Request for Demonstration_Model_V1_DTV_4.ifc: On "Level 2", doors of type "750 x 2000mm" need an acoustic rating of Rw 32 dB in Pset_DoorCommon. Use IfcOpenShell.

First a look at what the model holds.

```python
import ifcopenshell
import ifcopenshell.util.element

model = ifcopenshell.open("Demonstration_Model_V1_DTV_4.ifc")
print(model.schema)
storey = next(s for s in model.by_type("IfcBuildingStorey") if s.Name == "Level 2")
doors = [e for e in ifcopenshell.util.element.get_decomposition(storey) if e.is_a("IfcDoor")]
seen = {}
for e in doors:
    element_type = ifcopenshell.util.element.get_type(e)
    key = (element_type.Name if element_type != e and element_type else None, ifcopenshell.util.element.get_pset(e, "Pset_DoorCommon", "AcousticRating"))
    seen[key] = seen.get(key, 0) + 1
for (name, value), count in sorted(seen.items(), key=str):
    print(count, "x", name, "|", value)
```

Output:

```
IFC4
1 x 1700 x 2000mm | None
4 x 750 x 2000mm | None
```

```python
import ifcopenshell
import ifcopenshell.api.pset
import ifcopenshell.util.element

model = ifcopenshell.open("Demonstration_Model_V1_DTV_4.ifc")

storey = next(s for s in model.by_type("IfcBuildingStorey") if s.Name == "Level 2")
doors = [e for e in ifcopenshell.util.element.get_decomposition(storey) if e.is_a("IfcDoor")]

count = 0
for e in doors:
    element_type = ifcopenshell.util.element.get_type(e)
    if element_type in (None, e) or element_type.Name != "750 x 2000mm":
        continue
    # add_pset returns the element's existing set when there is one.
    pset = ifcopenshell.api.pset.add_pset(model, product=e, name="Pset_DoorCommon")
    ifcopenshell.api.pset.edit_pset(model, pset=pset, properties={"AcousticRating": "Rw 32 dB"})
    count += 1

print(count, "doors updated")

model.write("Demonstration_Model_V1_DTV_4_rev.ifc")
```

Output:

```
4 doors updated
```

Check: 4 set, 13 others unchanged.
